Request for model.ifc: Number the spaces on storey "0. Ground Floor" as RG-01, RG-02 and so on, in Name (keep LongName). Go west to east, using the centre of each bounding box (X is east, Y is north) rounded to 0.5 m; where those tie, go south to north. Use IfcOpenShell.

First a look at what the model holds.

```python
import ifcopenshell
import ifcopenshell.util.element
import ifcopenshell.util.placement

model = ifcopenshell.open("model.ifc")
print(model.schema)
storey = next(s for s in model.by_type("IfcBuildingStorey") if s.Name == "0. Ground Floor")
spaces = [e for e in ifcopenshell.util.element.get_decomposition(storey) if e.is_a("IfcSpace")]
for e in sorted(spaces, key=lambda e: e.id()):
    origin = ifcopenshell.util.placement.get_local_placement(e.ObjectPlacement)[:3, 3]
    print(e.id(), e.Name, e.LongName, origin.round(2) + 0.0, sep=" | ")
```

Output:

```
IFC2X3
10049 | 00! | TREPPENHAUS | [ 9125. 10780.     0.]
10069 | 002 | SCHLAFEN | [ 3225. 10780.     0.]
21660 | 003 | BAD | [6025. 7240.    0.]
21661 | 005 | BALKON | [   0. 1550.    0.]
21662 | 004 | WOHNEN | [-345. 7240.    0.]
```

```python
import ifcopenshell
import ifcopenshell.geom
import ifcopenshell.util.element
import ifcopenshell.util.shape

model = ifcopenshell.open("model.ifc")
settings = ifcopenshell.geom.settings()
settings.set("use-world-coords", True)


def centre(element):
    shape = ifcopenshell.geom.create_shape(settings, element)
    return ifcopenshell.util.shape.get_bbox_centroid(shape.geometry)


storey = next(s for s in model.by_type("IfcBuildingStorey") if s.Name == "0. Ground Floor")
spaces = [e for e in ifcopenshell.util.element.get_decomposition(storey) if e.is_a("IfcSpace")]

# Insertion points can sit at a corner or the storey origin, so sort by the geometry (in metres).
centres = {e: centre(e) for e in spaces}
spaces.sort(key=lambda e: (round(centres[e][0] / 0.5), centres[e][1]))

for i, e in enumerate(spaces, start=1):
    number = f"RG-{i:02d}"
    e.Name = number
    print(e.id(), number)

model.write("model_v2.ifc")
```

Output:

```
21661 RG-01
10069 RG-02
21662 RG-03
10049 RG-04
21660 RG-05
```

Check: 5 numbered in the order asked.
